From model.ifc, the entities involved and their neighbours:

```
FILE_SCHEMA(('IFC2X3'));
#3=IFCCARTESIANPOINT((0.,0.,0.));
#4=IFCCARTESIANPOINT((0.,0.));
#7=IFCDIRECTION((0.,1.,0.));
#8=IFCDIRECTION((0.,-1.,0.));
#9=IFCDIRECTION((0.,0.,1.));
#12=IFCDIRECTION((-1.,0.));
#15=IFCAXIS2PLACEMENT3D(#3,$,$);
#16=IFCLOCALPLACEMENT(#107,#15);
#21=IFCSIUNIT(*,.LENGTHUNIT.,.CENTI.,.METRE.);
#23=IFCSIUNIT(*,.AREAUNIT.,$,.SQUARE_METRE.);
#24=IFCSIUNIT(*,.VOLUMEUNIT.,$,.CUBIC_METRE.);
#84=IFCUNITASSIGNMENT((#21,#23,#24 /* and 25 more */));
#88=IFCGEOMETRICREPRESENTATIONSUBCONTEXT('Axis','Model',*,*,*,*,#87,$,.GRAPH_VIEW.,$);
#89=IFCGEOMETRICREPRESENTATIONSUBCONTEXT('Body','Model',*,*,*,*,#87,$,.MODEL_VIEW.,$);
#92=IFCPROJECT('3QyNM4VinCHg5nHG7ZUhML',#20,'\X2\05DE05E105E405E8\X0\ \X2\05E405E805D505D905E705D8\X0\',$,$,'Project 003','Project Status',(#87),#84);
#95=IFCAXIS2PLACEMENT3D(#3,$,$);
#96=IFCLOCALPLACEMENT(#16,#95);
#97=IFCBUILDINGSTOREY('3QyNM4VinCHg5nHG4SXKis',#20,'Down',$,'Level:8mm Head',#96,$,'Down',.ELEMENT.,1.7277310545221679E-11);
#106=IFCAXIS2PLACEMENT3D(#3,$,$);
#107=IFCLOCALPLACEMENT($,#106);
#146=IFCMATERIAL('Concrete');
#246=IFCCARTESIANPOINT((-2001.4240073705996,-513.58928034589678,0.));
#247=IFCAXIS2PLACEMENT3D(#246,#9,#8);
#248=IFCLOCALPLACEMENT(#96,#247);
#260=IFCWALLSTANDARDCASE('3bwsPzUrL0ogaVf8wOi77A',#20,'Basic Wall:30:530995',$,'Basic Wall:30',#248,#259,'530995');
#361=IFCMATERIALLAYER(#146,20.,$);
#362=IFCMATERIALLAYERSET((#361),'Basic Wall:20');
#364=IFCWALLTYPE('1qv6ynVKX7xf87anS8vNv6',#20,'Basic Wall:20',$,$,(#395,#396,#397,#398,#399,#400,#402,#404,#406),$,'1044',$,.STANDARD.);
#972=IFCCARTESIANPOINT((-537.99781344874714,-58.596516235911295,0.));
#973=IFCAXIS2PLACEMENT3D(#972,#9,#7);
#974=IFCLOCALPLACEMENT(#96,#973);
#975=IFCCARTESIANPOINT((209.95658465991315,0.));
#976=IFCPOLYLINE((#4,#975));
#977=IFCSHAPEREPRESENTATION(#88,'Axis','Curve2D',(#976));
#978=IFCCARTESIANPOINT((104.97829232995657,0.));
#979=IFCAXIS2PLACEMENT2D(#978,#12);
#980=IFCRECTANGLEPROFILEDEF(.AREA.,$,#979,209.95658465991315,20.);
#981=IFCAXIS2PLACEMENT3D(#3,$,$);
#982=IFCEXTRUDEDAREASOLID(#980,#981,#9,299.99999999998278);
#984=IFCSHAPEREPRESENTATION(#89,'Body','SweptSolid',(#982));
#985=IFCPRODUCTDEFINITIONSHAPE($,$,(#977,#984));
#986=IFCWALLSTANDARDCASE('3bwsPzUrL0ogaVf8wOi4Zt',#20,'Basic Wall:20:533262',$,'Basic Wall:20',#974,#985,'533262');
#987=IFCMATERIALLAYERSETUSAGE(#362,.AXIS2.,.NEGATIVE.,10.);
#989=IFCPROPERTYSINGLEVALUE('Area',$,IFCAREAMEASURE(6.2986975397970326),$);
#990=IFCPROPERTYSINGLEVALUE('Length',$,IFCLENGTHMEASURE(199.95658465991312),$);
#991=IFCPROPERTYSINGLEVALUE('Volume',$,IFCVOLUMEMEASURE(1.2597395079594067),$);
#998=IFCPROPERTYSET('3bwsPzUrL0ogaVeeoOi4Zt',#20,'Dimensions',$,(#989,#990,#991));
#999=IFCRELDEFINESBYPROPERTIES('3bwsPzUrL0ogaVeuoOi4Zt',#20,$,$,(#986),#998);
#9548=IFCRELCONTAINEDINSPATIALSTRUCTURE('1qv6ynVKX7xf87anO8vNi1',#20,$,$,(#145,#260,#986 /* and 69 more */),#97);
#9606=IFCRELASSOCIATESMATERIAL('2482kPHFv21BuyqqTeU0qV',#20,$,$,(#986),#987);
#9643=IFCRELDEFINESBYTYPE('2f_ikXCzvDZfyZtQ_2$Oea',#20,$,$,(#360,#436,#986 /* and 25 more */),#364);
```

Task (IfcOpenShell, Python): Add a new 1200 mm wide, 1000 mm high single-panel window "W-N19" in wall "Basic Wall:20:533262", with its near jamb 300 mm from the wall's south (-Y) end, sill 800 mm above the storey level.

```python
import numpy as np
import ifcopenshell
import ifcopenshell.api.feature
import ifcopenshell.api.geometry
import ifcopenshell.api.pset
import ifcopenshell.api.root
import ifcopenshell.api.spatial
import ifcopenshell.api.type
import ifcopenshell.geom
import ifcopenshell.util.element
import ifcopenshell.util.placement
import ifcopenshell.util.representation
import ifcopenshell.util.shape
import ifcopenshell.util.unit

model = ifcopenshell.open("model.ifc")
unit_scale = ifcopenshell.util.unit.calculate_unit_scale(model)
area_scale = ifcopenshell.util.unit.calculate_unit_scale(model, "AREAUNIT")
volume_scale = ifcopenshell.util.unit.calculate_unit_scale(model, "VOLUMEUNIT")
settings = ifcopenshell.geom.settings()


def volume(element):
    """Net volume in cubic metres, openings subtracted."""
    shape = ifcopenshell.geom.create_shape(settings, element)
    return ifcopenshell.util.shape.get_volume(shape.geometry)


wall = model.by_guid("3bwsPzUrL0ogaVf8wOi4Zt")
storey = ifcopenshell.util.element.get_container(wall, ifc_class="IfcBuildingStorey")
context = ifcopenshell.util.representation.get_context(model, "Model", "Body", "MODEL_VIEW")
before = volume(wall)

width, height, from_end, sill = 1.2, 1, 0.3, 0.8  # metres

# The wall runs along its own X axis, and the end named is its -X end.
wall_shape = ifcopenshell.geom.create_shape(settings, wall)
x, y, z = ifcopenshell.util.shape.get_vertices(wall_shape.geometry).T
start = x.min() + from_end
face, thickness = float(y.min()), float(y.max() - y.min())
wall_matrix = ifcopenshell.util.placement.get_local_placement(wall.ObjectPlacement)
level = ifcopenshell.util.placement.get_local_placement(storey.ObjectPlacement)[2, 3]


def in_wall(x, y):
    """Placement at x, y metres in the wall's axes, at sill height."""
    matrix = wall_matrix.copy()
    matrix[:, 3] = wall_matrix @ np.array([x / unit_scale, y / unit_scale, 0.0, 1.0])
    matrix[2, 3] = level + sill / unit_scale
    return matrix


# Opening: a box that overshoots both wall faces by 50 mm.
opening = ifcopenshell.api.root.create_entity(model, ifc_class="IfcOpeningElement")
box = ifcopenshell.api.geometry.add_wall_representation(
    model, context=context, length=width, height=height, thickness=thickness + 0.1
)
ifcopenshell.api.geometry.assign_representation(model, product=opening, representation=box)
ifcopenshell.api.geometry.edit_object_placement(model, product=opening, matrix=in_wall(start, face - 0.05), is_si=False)
ifcopenshell.api.feature.add_feature(model, feature=opening, element=wall)

window = ifcopenshell.api.root.create_entity(model, ifc_class="IfcWindow", name="W-N19")
window.OverallWidth, window.OverallHeight = width / unit_scale, height / unit_scale
body = ifcopenshell.api.geometry.add_window_representation(
    model,
    context=context,
    overall_width=window.OverallWidth,
    overall_height=window.OverallHeight,
    partition_type="SINGLE_PANEL",
)
ifcopenshell.api.geometry.assign_representation(model, product=window, representation=body)
ifcopenshell.api.spatial.assign_container(model, products=[window], relating_structure=storey)
fills = ifcopenshell.api.feature.add_filling(model, opening=opening, element=window)
fills.OwnerHistory = window.OwnerHistory  # required in IFC2X3

# IFC2X3 keeps the operation on the window style.
style = ifcopenshell.api.root.create_entity(model, ifc_class="IfcWindowStyle", name="W-N19")
style.OperationType, style.ConstructionType = "SINGLE_PANEL", "NOTDEFINED"
style.ParameterTakesPrecedence = style.Sizeable = False
ifcopenshell.api.type.assign_type(model, related_objects=[window], relating_type=style)

# Centre the window in the wall's thickness.
ifcopenshell.api.geometry.edit_object_placement(model, product=window, matrix=in_wall(start, face), is_si=False)
window_shape = ifcopenshell.geom.create_shape(settings, window)
depth = ifcopenshell.util.shape.get_vertices(window_shape.geometry)[:, 1]
offset = face + thickness / 2 - (depth.min() + depth.max()) / 2
ifcopenshell.api.geometry.edit_object_placement(model, product=window, matrix=in_wall(start, offset), is_si=False)

after = volume(wall)

# Update the wall's stored quantities.
pset = model.by_id(ifcopenshell.util.element.get_pset(wall, "Dimensions", should_inherit=False)["id"])
ifcopenshell.api.pset.edit_pset(model, pset=pset, properties={
    "Area": model.create_entity("IfcAreaMeasure", after / thickness / area_scale),
    "Volume": model.create_entity("IfcVolumeMeasure", after / volume_scale),
})

print(f"wall volume {before:.3f} -> {after:.3f} m3")

model.write("model_updated.ifc")
```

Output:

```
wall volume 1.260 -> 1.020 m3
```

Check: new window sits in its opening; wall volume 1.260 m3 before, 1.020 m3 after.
